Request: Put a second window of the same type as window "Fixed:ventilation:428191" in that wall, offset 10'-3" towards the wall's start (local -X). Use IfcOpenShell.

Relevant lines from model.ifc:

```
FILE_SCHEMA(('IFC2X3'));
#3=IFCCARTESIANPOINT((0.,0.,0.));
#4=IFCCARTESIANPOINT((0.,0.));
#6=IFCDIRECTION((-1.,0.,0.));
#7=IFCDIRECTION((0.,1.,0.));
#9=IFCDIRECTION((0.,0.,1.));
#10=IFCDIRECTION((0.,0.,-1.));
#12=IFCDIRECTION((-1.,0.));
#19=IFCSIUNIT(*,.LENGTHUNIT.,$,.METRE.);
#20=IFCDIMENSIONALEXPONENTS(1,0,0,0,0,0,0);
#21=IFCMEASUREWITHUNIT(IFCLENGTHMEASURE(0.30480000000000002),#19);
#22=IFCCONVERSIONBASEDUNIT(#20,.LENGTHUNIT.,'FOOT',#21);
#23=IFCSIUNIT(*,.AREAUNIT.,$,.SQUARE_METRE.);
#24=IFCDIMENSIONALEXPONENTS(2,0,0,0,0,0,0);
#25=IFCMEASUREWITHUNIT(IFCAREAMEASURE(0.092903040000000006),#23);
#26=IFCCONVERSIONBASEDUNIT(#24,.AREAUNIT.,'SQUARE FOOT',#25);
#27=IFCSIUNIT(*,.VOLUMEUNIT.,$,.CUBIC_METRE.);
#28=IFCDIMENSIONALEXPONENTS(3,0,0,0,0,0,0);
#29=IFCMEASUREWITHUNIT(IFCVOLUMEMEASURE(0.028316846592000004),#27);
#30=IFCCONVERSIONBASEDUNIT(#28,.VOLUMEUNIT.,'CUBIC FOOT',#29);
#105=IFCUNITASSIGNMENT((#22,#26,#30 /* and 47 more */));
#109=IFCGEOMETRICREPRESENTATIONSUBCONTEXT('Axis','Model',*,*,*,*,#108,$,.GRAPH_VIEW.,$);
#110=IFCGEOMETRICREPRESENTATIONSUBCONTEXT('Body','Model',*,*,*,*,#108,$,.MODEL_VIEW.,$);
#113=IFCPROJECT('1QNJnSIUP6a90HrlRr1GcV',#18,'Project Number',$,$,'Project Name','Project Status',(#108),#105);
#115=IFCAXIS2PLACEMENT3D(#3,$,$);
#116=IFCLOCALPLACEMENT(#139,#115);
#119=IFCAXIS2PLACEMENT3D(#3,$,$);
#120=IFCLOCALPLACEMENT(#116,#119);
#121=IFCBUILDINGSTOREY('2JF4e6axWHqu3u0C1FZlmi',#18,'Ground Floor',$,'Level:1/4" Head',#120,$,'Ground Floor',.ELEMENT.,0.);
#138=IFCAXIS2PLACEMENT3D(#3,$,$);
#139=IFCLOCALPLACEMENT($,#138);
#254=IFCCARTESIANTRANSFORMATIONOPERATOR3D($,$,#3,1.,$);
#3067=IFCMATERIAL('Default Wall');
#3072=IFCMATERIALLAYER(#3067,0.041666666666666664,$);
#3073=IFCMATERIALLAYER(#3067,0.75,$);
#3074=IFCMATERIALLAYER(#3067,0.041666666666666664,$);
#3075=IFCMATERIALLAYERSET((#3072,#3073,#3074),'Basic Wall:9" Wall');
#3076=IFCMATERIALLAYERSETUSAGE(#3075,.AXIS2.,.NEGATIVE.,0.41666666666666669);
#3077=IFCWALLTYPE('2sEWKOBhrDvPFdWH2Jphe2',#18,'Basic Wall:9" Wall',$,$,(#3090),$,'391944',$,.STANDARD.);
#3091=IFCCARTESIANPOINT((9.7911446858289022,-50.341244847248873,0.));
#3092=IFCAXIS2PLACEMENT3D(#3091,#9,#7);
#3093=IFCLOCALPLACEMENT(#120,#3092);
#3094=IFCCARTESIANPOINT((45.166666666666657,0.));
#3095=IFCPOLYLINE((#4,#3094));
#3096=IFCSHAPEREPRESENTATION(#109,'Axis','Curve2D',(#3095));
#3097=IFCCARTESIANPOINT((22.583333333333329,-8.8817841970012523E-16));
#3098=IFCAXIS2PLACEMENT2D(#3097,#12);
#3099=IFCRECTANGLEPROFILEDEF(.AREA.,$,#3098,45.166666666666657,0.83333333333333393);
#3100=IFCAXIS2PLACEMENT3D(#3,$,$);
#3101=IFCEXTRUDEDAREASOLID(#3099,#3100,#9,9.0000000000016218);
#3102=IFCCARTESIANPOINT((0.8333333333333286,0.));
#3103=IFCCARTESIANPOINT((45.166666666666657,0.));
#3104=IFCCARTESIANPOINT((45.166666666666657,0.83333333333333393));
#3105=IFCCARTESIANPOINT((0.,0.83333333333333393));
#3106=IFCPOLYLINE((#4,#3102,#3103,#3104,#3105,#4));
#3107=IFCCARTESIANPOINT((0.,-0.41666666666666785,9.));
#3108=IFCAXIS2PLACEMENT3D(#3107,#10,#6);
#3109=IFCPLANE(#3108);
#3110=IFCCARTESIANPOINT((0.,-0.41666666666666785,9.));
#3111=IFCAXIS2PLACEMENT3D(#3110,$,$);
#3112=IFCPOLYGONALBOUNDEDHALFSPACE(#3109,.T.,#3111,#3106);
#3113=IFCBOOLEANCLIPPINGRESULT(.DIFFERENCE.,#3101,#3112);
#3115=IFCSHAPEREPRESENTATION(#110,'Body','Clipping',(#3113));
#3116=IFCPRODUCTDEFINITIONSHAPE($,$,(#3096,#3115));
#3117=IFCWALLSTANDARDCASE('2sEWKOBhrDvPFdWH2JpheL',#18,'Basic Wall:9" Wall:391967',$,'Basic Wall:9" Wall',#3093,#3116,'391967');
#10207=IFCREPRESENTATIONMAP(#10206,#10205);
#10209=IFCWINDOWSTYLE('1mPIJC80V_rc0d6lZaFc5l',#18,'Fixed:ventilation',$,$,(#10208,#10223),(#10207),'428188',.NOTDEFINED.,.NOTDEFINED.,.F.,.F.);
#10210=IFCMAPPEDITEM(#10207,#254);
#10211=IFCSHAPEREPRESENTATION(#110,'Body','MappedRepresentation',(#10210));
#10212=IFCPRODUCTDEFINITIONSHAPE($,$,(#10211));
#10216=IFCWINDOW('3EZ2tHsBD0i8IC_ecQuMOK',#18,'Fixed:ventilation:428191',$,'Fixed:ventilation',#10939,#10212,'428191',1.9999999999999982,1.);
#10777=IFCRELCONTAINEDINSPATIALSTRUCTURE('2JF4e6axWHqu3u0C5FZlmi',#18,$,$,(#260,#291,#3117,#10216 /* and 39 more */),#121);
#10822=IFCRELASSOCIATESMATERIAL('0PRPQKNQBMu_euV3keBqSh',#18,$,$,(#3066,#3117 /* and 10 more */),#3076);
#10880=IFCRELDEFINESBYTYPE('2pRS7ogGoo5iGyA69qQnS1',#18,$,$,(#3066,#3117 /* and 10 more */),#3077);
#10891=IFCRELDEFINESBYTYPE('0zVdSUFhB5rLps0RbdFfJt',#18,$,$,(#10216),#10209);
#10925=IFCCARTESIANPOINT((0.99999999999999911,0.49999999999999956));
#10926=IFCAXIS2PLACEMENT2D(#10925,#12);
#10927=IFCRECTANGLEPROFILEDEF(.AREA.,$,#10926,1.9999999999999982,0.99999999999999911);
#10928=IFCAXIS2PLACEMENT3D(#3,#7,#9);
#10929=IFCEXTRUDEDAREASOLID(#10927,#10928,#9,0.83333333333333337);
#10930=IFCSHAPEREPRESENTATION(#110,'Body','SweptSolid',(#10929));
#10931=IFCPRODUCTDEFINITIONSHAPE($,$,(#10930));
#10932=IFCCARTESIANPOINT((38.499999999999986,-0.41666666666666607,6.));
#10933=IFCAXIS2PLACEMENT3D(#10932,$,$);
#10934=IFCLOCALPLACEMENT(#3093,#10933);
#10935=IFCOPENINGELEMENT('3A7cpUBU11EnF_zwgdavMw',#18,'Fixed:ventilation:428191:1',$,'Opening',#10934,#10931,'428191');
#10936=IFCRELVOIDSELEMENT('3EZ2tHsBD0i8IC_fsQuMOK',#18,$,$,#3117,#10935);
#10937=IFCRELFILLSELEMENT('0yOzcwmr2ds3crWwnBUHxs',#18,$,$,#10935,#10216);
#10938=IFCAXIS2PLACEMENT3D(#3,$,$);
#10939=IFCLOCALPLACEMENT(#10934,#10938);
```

```python
import ifcopenshell
import ifcopenshell.api.feature
import ifcopenshell.api.geometry
import ifcopenshell.api.root
import ifcopenshell.geom
import ifcopenshell.util.element
import ifcopenshell.util.placement
import ifcopenshell.util.shape
import ifcopenshell.util.unit

model = ifcopenshell.open("model.ifc")
unit_scale = ifcopenshell.util.unit.calculate_unit_scale(model)
settings = ifcopenshell.geom.settings()


def volume(element):
    """Net volume in cubic metres, openings subtracted."""
    shape = ifcopenshell.geom.create_shape(settings, element)
    return ifcopenshell.util.shape.get_volume(shape.geometry)


def reuse_history(source, copy):
    """copy_class also copies each property set's owner history, people and application; keep the originals."""
    for rel in copy.IsDefinedBy:
        if rel.is_a("IfcRelDefinesByProperties") and (history := rel.RelatingPropertyDefinition.OwnerHistory):
            rel.RelatingPropertyDefinition.OwnerHistory = source.OwnerHistory
            ifcopenshell.util.element.remove_deep2(model, history)


window = model.by_guid("3EZ2tHsBD0i8IC_ecQuMOK")
opening = window.FillsVoids[0].RelatingOpeningElement
wall = opening.VoidsElements[0].RelatingBuildingElement
before = volume(wall)
shift = ifcopenshell.util.placement.get_local_placement(wall.ObjectPlacement)[:3, 0] * -123 * 0.0254 / unit_scale

# copy_class copies the void relationship, type, container and properties, but no geometry.
new_opening = ifcopenshell.api.root.copy_class(model, product=opening)
new_opening.Representation = ifcopenshell.util.element.copy_deep(
    model, opening.Representation, exclude=["IfcGeometricRepresentationContext", "IfcRepresentationMap"]
)
new_opening.Name = "Fixed:ventilation"
new_opening.Tag = None
new_window = ifcopenshell.api.root.copy_class(model, product=window)
new_window.Representation = ifcopenshell.util.element.copy_deep(
    model, window.Representation, exclude=["IfcGeometricRepresentationContext", "IfcRepresentationMap"]
)
new_window.Name = "Fixed:ventilation"
new_window.Tag = None
reuse_history(window, new_window)
fills = ifcopenshell.api.feature.add_filling(model, opening=new_opening, element=new_window)
fills.OwnerHistory = new_window.OwnerHistory  # required in IFC2X3

for old, new in ((opening, new_opening), (window, new_window)):
    matrix = ifcopenshell.util.placement.get_local_placement(old.ObjectPlacement)
    matrix[:3, 3] += shift
    ifcopenshell.api.geometry.edit_object_placement(model, product=new, matrix=matrix, is_si=False)

after = volume(wall)

print(f"wall volume {before:.3f} -> {after:.3f} m3")

model.write("model-out.ifc")
```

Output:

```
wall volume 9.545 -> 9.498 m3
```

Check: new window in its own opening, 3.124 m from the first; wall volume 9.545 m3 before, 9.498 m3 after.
